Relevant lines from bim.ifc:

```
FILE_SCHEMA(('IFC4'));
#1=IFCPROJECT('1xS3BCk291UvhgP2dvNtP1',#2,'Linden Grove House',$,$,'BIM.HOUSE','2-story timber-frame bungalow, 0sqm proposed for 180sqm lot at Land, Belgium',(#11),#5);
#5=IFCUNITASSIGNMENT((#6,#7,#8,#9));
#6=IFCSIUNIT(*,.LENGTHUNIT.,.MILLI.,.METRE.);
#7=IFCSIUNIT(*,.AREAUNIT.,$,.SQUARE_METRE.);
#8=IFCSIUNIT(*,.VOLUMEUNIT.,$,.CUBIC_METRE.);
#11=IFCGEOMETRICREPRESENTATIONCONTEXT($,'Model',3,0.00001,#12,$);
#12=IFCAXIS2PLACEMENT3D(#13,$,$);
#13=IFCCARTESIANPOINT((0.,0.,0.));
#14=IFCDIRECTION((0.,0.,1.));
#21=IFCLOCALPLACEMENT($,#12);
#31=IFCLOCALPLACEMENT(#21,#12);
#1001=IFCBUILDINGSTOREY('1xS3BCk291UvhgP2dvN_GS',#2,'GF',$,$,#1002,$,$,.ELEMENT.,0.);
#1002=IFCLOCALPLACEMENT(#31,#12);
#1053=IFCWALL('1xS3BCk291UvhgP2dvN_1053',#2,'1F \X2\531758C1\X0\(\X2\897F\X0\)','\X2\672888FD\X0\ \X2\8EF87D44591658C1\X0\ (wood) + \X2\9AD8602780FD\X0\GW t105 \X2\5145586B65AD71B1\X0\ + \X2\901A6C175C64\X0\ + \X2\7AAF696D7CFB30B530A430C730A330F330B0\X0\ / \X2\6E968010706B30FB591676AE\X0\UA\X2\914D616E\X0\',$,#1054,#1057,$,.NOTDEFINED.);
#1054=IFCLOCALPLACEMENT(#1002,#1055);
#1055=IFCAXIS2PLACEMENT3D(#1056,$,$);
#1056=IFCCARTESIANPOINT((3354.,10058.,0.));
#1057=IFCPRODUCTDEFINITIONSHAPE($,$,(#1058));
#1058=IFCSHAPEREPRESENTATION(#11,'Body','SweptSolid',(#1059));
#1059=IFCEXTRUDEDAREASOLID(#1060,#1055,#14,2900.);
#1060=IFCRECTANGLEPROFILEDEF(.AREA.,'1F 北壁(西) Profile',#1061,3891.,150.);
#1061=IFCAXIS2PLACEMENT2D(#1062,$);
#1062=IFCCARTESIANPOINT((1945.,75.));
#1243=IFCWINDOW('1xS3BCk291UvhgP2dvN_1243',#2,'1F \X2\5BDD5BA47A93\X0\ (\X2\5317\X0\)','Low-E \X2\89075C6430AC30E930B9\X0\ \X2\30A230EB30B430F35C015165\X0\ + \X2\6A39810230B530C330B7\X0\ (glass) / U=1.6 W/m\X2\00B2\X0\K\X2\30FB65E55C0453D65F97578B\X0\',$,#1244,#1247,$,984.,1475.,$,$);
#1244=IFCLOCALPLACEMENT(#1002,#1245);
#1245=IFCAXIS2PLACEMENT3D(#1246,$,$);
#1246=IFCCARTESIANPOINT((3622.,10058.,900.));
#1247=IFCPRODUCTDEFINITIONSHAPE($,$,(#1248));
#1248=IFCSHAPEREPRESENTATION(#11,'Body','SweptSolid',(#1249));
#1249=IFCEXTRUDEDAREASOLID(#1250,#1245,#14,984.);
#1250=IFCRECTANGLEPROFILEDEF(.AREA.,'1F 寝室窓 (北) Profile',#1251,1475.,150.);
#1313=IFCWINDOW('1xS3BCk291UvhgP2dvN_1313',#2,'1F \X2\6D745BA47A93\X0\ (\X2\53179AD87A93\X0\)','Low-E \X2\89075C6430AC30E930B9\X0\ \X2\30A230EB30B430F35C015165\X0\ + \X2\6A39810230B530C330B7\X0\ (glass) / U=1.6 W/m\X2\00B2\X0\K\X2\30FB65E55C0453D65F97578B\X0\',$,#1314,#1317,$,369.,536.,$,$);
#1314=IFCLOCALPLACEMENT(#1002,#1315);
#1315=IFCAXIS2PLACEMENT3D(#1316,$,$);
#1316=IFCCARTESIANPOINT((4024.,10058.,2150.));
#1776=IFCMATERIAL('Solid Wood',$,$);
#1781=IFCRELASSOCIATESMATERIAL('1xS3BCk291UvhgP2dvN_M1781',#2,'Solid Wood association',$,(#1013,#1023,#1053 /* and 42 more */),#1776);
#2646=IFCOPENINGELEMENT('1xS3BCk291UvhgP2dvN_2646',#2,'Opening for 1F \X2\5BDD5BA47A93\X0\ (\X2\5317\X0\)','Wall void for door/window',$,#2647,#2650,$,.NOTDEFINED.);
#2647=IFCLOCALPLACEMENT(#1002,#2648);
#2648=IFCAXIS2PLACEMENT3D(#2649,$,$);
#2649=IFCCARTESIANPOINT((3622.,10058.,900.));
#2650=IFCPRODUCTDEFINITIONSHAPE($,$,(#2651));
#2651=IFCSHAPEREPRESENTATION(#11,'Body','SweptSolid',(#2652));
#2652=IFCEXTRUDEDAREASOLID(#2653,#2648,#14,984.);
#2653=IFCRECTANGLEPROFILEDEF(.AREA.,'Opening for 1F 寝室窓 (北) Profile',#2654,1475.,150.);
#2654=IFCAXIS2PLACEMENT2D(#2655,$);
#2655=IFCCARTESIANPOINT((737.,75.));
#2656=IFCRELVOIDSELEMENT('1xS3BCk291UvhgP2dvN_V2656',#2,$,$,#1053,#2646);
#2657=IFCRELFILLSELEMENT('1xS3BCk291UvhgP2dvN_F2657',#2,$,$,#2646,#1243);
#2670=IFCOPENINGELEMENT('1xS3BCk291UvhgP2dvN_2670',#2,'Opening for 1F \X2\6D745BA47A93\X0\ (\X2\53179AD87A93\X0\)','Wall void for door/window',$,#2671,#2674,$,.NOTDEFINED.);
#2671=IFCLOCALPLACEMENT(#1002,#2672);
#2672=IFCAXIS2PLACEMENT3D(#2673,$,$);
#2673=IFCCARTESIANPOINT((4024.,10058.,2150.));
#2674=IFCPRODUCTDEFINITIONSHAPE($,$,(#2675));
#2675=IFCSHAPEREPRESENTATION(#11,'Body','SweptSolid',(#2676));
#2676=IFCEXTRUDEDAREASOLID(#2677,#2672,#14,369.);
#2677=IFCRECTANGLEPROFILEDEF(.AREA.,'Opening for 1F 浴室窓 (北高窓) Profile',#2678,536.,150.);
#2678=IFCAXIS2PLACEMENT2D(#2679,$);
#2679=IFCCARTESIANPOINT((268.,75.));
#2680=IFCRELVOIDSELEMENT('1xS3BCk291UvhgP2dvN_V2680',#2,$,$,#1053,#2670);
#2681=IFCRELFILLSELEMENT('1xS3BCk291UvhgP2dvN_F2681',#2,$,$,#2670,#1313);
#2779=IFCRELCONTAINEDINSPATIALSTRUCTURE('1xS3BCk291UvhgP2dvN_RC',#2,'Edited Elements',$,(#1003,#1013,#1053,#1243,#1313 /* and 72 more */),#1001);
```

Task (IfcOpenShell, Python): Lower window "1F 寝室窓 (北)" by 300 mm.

```python
import numpy as np
import ifcopenshell
import ifcopenshell.api.geometry
import ifcopenshell.util.placement
import ifcopenshell.util.unit

model = ifcopenshell.open("bim.ifc")
unit_scale = ifcopenshell.util.unit.calculate_unit_scale(model)

window = model.by_guid("1xS3BCk291UvhgP2dvN_1243")
opening = window.FillsVoids[0].RelatingOpeningElement
dz = -0.3 / unit_scale

shift = np.array([0.0, 0.0, dz])
# The window is not placed relative to its opening, so move both.
for product in (opening, window):
    matrix = ifcopenshell.util.placement.get_local_placement(product.ObjectPlacement)
    matrix[:3, 3] += shift
    ifcopenshell.api.geometry.edit_object_placement(model, product=product, matrix=matrix, is_si=False)

print(f"moved by {dz * unit_scale:+.3f} m")

model.write("bim_v2.ifc")
```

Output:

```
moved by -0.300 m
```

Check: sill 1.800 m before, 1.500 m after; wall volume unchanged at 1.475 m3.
